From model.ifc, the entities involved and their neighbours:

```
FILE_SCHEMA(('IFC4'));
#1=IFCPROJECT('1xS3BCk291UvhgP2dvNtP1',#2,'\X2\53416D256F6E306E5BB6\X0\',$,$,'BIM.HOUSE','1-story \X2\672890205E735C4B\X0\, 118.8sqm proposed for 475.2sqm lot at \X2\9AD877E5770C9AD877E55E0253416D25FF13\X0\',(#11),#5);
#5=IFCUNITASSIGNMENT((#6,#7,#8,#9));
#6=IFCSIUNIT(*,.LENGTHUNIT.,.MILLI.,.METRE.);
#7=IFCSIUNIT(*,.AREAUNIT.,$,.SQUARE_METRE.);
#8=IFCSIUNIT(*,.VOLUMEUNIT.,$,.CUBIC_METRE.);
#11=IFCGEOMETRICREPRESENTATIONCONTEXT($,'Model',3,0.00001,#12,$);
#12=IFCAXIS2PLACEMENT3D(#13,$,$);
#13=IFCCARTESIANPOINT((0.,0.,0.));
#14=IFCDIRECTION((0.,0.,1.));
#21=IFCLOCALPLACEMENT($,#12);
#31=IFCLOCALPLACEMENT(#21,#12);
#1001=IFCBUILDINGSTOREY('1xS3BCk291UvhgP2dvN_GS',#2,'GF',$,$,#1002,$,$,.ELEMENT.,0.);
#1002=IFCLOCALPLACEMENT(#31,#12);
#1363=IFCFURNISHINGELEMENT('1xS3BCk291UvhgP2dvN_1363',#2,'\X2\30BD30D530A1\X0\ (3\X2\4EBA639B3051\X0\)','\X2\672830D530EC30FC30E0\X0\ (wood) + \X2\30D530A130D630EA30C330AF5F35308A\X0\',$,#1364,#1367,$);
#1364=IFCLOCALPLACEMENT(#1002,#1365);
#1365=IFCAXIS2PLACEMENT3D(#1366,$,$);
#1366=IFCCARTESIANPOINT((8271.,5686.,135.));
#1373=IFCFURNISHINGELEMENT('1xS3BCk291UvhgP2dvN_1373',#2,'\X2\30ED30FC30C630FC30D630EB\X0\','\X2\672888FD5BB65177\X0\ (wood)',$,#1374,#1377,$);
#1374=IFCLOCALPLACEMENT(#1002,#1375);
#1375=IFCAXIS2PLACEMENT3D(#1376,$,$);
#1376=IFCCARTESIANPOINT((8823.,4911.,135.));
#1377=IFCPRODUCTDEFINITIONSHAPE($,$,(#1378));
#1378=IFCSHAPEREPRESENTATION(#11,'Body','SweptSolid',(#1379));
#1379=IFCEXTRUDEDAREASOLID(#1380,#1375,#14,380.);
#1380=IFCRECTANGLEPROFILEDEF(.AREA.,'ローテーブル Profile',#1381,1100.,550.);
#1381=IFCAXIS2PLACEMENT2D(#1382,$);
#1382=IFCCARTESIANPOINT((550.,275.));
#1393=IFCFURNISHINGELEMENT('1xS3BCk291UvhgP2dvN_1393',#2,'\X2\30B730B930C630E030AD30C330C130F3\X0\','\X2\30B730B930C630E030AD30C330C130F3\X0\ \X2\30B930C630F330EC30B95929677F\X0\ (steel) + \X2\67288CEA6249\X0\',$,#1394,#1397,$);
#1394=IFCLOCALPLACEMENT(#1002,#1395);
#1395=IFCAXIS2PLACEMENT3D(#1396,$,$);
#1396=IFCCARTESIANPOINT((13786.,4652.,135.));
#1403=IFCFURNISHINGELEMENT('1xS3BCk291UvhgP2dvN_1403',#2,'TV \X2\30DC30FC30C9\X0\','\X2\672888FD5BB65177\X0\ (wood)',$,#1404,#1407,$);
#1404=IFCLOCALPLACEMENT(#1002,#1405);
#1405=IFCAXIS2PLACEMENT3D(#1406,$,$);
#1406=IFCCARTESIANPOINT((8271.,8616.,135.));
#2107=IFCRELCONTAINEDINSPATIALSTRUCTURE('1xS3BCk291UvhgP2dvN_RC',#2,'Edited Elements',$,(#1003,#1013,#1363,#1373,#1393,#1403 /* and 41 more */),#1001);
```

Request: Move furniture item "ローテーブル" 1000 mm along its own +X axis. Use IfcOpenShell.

```python
import ifcopenshell
import ifcopenshell.api.geometry
import ifcopenshell.util.placement
import ifcopenshell.util.unit

model = ifcopenshell.open("model.ifc")
unit_scale = ifcopenshell.util.unit.calculate_unit_scale(model)

item = model.by_guid("1xS3BCk291UvhgP2dvN_1373")
matrix = ifcopenshell.util.placement.get_local_placement(item.ObjectPlacement)
matrix[:3, 3] += matrix[:3, 0] * 1 / unit_scale
ifcopenshell.api.geometry.edit_object_placement(model, product=item, matrix=matrix, is_si=False)

print(ifcopenshell.util.placement.get_local_placement(item.ObjectPlacement).round(3) + 0.0)

model.write("model_updated.ifc")
```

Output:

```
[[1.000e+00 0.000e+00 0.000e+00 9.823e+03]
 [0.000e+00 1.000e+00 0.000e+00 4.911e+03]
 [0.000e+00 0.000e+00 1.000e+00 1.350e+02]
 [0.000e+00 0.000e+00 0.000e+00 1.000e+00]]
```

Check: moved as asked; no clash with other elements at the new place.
